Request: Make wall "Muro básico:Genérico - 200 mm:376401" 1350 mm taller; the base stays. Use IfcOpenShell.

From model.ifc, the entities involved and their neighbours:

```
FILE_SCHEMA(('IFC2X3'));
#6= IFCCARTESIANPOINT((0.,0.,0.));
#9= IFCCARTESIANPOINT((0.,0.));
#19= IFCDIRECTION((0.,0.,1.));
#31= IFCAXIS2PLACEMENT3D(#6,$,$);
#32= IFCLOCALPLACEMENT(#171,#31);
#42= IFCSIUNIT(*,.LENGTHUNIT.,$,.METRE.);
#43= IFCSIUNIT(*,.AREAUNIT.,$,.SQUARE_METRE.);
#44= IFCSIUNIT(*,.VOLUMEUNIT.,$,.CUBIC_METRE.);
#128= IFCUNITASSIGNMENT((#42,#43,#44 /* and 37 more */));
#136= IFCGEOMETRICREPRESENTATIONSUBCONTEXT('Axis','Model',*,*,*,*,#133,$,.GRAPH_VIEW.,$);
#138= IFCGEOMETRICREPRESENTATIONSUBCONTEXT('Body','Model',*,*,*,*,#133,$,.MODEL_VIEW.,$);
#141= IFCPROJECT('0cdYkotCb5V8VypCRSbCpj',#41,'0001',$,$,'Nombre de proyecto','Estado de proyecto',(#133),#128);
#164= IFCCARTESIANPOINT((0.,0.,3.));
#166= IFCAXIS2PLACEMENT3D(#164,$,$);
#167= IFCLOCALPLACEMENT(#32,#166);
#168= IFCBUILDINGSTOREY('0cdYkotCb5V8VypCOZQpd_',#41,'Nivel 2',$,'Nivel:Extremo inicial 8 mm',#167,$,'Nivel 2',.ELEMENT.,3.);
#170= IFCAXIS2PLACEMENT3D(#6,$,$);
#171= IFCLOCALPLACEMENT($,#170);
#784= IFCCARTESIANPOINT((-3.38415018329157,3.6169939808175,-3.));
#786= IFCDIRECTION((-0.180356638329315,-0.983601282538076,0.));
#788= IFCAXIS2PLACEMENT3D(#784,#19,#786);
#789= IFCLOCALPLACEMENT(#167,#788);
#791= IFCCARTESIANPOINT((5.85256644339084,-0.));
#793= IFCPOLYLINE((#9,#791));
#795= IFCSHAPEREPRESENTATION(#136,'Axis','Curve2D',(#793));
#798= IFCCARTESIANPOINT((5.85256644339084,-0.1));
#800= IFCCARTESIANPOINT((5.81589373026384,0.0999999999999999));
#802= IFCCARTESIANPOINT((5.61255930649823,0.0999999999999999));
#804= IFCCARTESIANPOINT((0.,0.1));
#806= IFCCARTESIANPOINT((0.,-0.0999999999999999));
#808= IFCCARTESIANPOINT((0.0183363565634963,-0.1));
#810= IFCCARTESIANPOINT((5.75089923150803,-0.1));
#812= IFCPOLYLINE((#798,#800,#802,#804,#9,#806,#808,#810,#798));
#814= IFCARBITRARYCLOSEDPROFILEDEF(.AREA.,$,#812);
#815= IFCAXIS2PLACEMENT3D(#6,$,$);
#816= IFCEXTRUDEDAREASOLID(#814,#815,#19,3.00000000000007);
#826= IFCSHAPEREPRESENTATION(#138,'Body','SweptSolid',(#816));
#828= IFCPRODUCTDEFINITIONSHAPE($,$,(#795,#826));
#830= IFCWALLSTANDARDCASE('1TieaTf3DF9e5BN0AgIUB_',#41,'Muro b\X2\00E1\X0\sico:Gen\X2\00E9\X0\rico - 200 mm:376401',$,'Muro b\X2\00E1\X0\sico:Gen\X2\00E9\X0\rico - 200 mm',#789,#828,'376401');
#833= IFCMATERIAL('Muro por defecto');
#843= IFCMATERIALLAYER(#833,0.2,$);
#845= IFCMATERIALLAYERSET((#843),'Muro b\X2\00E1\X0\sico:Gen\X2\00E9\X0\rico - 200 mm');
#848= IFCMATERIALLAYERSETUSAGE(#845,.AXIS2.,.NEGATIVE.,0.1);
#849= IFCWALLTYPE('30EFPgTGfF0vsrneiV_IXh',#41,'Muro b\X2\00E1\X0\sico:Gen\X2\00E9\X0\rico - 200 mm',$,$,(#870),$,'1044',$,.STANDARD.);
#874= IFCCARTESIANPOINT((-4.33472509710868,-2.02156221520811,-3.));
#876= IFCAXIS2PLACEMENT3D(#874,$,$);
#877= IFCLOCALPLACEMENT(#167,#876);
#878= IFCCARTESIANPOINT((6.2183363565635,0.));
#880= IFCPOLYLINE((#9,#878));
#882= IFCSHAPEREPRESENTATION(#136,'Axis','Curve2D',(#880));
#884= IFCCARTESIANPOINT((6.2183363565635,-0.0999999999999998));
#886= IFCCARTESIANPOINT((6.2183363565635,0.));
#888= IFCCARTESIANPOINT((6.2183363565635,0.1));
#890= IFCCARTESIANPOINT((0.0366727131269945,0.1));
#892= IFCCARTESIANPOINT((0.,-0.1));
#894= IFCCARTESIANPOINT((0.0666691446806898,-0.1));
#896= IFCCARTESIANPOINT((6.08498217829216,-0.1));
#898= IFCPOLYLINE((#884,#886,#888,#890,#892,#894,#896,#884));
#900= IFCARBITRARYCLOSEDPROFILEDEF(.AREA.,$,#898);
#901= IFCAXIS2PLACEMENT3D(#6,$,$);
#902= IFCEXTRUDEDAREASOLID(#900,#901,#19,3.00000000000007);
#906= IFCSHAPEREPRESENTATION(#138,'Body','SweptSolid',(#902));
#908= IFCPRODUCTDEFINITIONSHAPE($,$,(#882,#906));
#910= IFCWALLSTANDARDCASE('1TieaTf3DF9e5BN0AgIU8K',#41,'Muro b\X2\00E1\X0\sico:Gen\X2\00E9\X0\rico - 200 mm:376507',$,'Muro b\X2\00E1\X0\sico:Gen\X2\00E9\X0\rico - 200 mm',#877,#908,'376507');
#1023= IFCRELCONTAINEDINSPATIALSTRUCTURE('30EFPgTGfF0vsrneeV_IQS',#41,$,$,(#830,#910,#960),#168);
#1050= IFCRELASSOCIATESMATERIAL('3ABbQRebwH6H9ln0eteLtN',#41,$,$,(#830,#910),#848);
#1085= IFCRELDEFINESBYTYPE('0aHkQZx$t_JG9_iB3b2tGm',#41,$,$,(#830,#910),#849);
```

```python
import ifcopenshell
import ifcopenshell.geom
import ifcopenshell.util.representation
import ifcopenshell.util.shape

model = ifcopenshell.open("model.ifc")
settings = ifcopenshell.geom.settings()


def volume(element):
    """Net volume in cubic metres, openings subtracted."""
    shape = ifcopenshell.geom.create_shape(settings, element)
    return ifcopenshell.util.shape.get_volume(shape.geometry)


wall = model.by_guid("1TieaTf3DF9e5BN0AgIUB_")
before = volume(wall)

body = ifcopenshell.util.representation.get_representation(wall, "Model", "Body")
solid = body.Items[0]
old_height = solid.Depth
solid.Depth += 1.35
after = volume(wall)

print(f"height {old_height:g} -> {solid.Depth:g}, volume {before:.3f} -> {after:.3f} m3")

model.write("model_updated.ifc")
```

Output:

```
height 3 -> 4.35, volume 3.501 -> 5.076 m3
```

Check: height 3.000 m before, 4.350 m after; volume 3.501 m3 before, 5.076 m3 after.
